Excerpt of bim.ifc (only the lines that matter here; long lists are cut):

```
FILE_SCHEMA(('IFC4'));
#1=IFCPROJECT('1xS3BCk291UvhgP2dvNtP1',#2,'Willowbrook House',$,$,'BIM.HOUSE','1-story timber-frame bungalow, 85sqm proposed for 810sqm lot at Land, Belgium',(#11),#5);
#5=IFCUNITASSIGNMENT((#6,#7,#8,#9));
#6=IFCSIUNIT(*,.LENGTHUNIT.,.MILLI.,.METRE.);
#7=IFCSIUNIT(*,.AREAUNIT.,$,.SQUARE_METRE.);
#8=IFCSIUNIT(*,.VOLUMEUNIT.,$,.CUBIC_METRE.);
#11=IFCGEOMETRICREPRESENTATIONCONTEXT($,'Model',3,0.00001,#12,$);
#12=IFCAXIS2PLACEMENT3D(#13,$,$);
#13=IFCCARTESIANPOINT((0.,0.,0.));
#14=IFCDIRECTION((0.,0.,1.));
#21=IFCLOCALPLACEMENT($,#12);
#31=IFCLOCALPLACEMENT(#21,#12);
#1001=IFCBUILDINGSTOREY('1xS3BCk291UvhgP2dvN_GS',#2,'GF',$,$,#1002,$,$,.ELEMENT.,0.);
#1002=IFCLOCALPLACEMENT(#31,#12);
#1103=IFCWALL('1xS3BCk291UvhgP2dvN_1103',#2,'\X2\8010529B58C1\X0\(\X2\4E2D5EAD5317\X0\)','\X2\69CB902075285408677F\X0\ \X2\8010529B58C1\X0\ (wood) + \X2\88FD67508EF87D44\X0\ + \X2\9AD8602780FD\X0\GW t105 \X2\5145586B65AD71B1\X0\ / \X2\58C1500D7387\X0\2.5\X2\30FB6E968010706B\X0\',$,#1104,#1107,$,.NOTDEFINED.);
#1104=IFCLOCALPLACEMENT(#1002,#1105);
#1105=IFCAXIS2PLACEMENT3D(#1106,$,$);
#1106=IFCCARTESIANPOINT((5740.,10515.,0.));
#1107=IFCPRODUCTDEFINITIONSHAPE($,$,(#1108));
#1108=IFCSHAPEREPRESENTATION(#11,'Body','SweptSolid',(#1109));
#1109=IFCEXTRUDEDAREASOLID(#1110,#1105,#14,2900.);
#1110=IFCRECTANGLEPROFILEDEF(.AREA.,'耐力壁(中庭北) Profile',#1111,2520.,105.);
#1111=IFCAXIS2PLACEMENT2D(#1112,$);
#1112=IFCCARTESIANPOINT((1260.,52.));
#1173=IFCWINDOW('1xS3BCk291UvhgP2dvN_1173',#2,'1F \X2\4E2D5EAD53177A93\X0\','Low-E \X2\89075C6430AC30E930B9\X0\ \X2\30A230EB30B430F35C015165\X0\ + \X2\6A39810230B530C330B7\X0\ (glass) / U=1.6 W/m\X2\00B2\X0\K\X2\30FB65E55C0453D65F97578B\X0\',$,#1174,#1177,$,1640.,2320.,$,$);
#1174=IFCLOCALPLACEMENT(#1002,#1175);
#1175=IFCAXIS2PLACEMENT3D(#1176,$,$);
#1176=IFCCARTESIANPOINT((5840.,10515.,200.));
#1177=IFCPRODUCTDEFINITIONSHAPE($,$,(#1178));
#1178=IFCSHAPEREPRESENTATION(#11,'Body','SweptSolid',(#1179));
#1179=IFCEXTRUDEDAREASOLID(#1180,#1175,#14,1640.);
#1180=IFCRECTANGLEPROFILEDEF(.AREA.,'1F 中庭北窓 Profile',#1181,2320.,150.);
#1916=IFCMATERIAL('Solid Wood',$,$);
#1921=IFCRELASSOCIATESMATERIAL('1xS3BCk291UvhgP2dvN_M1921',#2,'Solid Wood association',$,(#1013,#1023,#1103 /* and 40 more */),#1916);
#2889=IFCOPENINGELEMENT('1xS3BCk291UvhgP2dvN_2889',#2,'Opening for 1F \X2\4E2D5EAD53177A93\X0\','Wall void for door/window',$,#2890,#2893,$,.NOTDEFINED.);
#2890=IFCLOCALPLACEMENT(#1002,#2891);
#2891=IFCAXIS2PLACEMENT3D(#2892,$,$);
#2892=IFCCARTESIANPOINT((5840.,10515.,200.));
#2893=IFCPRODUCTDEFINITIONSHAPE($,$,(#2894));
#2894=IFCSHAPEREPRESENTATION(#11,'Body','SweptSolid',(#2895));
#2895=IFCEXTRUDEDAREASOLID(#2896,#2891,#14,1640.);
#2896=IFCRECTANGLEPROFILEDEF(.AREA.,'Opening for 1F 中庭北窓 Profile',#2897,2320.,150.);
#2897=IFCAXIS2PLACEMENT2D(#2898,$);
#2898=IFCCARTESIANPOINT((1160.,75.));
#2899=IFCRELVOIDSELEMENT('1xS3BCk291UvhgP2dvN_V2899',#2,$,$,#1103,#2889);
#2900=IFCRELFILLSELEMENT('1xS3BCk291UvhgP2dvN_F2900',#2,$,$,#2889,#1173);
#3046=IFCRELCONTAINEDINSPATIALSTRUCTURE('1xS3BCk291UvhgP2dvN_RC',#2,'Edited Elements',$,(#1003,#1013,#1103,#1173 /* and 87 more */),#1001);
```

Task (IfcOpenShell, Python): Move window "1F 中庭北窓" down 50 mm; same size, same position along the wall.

```python
import numpy as np
import ifcopenshell
import ifcopenshell.api.geometry
import ifcopenshell.util.placement
import ifcopenshell.util.unit

model = ifcopenshell.open("bim.ifc")
unit_scale = ifcopenshell.util.unit.calculate_unit_scale(model)

window = model.by_id(1173)
opening = window.FillsVoids[0].RelatingOpeningElement
dz = -50.0

shift = np.array([0.0, 0.0, dz])
# The window is not placed relative to its opening, so move both.
for product in (opening, window):
    matrix = ifcopenshell.util.placement.get_local_placement(product.ObjectPlacement)
    matrix[:3, 3] += shift
    ifcopenshell.api.geometry.edit_object_placement(model, product=product, matrix=matrix, is_si=False)

print(f"moved by {dz * unit_scale:+.3f} m")

model.write("bim_updated.ifc")
```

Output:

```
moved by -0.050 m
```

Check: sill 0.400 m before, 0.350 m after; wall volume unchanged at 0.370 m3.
